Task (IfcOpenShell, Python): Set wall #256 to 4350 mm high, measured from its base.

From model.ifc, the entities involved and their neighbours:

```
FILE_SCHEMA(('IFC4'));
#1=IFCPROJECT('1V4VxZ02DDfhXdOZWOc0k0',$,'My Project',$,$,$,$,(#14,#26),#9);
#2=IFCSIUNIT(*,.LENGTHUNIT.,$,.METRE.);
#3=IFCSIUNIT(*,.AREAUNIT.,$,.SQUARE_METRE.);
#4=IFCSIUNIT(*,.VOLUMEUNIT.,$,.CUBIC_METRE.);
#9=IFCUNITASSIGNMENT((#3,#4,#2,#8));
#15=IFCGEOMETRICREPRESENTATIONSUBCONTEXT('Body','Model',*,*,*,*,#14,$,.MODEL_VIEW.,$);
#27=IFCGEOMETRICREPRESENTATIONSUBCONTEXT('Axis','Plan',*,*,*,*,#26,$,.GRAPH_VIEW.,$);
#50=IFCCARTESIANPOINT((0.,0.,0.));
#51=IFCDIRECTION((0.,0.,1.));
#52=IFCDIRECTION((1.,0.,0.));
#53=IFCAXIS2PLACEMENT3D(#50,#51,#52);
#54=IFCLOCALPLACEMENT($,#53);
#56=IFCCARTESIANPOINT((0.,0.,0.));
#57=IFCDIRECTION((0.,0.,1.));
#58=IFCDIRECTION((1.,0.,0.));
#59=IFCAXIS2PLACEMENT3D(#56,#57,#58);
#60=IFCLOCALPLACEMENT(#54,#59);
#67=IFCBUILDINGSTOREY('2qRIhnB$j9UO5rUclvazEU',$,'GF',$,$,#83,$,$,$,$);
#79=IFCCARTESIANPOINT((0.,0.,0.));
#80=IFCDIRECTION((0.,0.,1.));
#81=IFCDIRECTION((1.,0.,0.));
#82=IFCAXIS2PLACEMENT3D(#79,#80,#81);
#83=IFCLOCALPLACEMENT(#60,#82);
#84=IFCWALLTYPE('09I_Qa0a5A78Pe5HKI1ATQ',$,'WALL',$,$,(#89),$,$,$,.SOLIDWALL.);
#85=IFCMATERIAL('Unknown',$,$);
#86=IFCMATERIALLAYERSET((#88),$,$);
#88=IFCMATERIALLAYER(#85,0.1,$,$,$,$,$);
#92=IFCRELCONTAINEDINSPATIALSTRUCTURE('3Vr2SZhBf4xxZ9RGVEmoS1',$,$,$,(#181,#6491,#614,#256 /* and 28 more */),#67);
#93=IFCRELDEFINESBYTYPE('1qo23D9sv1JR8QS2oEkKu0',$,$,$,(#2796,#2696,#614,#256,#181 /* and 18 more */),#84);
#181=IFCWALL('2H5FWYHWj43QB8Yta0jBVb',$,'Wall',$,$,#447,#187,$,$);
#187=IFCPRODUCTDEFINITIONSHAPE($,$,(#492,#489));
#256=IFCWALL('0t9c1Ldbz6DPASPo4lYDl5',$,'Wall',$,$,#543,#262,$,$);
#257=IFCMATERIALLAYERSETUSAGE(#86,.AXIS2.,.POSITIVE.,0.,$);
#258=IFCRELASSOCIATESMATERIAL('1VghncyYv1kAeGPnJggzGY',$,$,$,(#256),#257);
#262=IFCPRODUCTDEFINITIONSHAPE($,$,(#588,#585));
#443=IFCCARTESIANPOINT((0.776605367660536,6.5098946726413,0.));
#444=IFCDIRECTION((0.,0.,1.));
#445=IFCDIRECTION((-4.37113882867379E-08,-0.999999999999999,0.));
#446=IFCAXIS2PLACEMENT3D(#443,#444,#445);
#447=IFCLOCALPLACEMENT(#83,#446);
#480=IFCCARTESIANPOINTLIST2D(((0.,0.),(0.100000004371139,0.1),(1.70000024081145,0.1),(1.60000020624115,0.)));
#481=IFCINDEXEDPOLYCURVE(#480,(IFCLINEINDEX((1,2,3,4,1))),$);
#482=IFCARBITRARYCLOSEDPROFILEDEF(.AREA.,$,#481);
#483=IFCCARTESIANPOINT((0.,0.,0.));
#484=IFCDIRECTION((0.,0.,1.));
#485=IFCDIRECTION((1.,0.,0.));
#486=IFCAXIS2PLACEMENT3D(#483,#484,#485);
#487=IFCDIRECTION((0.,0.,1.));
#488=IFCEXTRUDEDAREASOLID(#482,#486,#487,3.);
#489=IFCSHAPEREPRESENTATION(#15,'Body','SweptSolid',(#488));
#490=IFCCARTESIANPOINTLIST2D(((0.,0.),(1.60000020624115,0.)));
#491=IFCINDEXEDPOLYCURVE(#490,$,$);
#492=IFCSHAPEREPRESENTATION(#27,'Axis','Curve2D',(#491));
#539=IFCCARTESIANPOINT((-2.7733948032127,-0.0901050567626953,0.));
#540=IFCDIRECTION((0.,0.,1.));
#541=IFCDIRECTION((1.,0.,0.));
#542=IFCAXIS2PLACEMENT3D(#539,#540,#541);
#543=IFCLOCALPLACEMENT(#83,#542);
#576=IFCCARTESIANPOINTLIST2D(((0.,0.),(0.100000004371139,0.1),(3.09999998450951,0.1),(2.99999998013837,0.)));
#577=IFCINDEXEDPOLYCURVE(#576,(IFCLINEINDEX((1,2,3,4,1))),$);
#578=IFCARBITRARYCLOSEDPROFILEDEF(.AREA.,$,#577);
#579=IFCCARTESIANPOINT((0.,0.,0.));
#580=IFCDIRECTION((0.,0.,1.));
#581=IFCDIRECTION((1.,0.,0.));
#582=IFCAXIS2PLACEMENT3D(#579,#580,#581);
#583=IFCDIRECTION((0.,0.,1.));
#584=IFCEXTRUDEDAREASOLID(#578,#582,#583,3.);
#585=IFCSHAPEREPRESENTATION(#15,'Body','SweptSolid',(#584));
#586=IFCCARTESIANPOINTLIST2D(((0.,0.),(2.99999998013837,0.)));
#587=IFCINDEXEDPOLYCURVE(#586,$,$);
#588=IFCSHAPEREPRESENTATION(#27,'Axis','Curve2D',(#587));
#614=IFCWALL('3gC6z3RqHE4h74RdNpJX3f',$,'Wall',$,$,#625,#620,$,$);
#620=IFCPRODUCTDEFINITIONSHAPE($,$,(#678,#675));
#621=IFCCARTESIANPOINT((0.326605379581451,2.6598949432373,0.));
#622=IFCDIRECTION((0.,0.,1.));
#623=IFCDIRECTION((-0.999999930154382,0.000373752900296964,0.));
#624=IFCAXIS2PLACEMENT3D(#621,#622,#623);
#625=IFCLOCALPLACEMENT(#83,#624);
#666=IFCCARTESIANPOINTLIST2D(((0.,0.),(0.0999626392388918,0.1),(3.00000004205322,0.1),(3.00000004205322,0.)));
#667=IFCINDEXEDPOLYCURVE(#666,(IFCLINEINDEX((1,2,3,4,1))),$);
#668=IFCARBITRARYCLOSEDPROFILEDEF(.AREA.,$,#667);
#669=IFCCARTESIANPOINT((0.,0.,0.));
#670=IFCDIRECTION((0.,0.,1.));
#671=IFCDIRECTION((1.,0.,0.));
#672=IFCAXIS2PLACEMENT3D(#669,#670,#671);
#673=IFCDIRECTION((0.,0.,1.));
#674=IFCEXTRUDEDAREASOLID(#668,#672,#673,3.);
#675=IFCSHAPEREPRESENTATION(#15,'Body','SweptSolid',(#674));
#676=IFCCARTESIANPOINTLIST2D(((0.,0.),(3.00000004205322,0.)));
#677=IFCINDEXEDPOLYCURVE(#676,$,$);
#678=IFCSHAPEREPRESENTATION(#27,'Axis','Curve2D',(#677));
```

```python
import ifcopenshell
import ifcopenshell.geom
import ifcopenshell.util.representation
import ifcopenshell.util.shape
import ifcopenshell.util.unit

model = ifcopenshell.open("model.ifc")
unit_scale = ifcopenshell.util.unit.calculate_unit_scale(model)
settings = ifcopenshell.geom.settings()


def volume(element):
    """Net volume in cubic metres, openings subtracted."""
    shape = ifcopenshell.geom.create_shape(settings, element)
    return ifcopenshell.util.shape.get_volume(shape.geometry)


wall = model.by_guid("0t9c1Ldbz6DPASPo4lYDl5")
before = volume(wall)

body = ifcopenshell.util.representation.get_representation(wall, "Model", "Body")
solid = body.Items[0]
old_height = solid.Depth
solid.Depth = 4.35 / unit_scale
after = volume(wall)

print(f"height {old_height:g} -> {solid.Depth:g}, volume {before:.3f} -> {after:.3f} m3")

model.write("model_edited.ifc")
```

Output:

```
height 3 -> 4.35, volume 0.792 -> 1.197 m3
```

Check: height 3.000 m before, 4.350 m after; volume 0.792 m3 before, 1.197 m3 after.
